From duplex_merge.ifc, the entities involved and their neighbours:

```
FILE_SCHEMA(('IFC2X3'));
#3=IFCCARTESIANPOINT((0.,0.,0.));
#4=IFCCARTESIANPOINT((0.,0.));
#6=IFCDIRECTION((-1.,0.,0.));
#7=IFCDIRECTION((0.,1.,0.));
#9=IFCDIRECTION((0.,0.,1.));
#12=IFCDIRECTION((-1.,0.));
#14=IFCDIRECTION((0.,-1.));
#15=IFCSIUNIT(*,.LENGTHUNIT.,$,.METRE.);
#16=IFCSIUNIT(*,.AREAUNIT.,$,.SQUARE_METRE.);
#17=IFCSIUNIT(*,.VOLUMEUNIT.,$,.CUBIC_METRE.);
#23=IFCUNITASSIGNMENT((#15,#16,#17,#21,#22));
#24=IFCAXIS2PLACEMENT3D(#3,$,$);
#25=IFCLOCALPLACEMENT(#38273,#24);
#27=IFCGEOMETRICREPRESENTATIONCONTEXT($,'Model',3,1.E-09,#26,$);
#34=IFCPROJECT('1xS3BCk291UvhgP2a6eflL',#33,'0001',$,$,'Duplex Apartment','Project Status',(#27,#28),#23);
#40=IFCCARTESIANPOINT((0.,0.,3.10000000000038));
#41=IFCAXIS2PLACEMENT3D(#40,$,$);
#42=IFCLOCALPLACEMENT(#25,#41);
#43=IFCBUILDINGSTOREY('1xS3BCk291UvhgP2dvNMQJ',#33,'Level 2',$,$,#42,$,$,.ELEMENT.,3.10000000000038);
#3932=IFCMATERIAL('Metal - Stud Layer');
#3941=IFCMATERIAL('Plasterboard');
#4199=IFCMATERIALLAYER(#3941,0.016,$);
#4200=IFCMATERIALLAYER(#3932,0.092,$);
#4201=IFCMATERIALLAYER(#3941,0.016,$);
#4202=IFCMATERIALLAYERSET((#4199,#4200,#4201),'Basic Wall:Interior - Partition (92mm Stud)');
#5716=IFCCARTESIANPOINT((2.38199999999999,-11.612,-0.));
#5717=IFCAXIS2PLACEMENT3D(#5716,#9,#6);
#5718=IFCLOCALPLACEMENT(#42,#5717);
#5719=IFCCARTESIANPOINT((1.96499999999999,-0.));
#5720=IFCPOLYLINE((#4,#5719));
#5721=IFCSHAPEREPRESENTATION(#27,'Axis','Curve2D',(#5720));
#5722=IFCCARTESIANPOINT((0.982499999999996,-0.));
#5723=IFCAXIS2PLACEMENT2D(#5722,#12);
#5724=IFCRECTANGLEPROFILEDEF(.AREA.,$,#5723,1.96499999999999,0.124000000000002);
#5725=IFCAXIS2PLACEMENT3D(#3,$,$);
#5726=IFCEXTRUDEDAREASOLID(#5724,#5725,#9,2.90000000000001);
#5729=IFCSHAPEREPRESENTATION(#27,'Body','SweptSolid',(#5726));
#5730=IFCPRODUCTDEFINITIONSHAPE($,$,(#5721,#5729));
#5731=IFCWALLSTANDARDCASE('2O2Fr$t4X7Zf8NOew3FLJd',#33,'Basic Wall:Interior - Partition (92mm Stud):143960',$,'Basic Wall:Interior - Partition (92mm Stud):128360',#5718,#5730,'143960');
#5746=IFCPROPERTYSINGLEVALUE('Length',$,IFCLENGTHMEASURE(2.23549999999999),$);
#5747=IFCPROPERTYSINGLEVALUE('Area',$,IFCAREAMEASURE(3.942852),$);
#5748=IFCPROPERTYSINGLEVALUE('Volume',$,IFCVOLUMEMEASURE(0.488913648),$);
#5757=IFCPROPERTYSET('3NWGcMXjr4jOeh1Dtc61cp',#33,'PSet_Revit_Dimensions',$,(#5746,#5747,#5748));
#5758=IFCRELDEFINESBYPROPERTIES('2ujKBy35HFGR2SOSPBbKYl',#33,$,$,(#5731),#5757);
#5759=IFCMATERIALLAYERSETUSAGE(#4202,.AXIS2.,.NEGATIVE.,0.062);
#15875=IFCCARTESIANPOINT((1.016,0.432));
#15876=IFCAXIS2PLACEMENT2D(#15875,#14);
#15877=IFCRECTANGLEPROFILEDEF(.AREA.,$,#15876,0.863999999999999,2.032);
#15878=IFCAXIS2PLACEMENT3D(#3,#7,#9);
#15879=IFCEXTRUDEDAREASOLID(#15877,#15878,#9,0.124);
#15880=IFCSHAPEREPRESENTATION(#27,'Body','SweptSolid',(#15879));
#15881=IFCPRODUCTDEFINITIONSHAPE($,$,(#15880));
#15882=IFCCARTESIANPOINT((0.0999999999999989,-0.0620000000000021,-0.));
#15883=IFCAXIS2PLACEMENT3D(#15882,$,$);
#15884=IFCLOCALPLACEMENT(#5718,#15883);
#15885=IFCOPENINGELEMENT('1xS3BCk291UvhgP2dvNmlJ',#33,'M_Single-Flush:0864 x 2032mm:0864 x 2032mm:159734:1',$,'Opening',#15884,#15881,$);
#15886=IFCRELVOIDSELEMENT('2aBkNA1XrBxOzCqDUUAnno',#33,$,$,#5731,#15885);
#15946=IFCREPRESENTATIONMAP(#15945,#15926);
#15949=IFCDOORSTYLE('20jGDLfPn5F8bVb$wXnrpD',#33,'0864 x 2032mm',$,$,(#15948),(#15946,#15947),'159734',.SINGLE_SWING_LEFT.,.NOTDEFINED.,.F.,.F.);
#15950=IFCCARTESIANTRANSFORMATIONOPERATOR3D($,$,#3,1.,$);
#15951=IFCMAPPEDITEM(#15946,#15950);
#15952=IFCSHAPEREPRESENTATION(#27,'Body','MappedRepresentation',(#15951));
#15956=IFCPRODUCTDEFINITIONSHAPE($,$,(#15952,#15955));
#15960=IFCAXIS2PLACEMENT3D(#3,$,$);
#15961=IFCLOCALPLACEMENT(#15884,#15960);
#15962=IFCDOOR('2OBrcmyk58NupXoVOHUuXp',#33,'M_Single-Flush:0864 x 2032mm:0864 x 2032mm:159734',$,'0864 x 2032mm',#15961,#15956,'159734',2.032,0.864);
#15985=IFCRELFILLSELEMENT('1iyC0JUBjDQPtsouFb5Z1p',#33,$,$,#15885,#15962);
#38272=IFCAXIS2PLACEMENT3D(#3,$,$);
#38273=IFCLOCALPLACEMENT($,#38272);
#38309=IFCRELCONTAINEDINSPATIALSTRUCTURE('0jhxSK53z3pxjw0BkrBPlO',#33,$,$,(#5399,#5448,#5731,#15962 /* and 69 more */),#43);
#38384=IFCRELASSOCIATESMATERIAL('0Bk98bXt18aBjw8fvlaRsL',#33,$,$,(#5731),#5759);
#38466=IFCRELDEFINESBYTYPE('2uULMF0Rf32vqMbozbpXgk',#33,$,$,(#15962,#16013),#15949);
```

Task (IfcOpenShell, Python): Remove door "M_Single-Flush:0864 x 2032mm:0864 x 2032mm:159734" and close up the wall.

```python
import ifcopenshell
import ifcopenshell.api.feature
import ifcopenshell.api.pset
import ifcopenshell.api.root
import ifcopenshell.geom
import ifcopenshell.util.element
import ifcopenshell.util.shape
import ifcopenshell.util.unit

model = ifcopenshell.open("duplex_merge.ifc")
area_scale = ifcopenshell.util.unit.calculate_unit_scale(model, "AREAUNIT")
volume_scale = ifcopenshell.util.unit.calculate_unit_scale(model, "VOLUMEUNIT")
settings = ifcopenshell.geom.settings()


def volume(element):
    """Net volume in cubic metres, openings subtracted."""
    shape = ifcopenshell.geom.create_shape(settings, element)
    return ifcopenshell.util.shape.get_volume(shape.geometry)


door = model.by_id(15962)
opening = door.FillsVoids[0].RelatingOpeningElement
wall = opening.VoidsElements[0].RelatingBuildingElement
before = volume(wall)

ifcopenshell.api.root.remove_product(model, product=door)
ifcopenshell.api.feature.remove_feature(model, feature=opening)

after = volume(wall)
thickness = 0.124  # wall thickness in metres

# Update the wall's stored quantities.
pset = model.by_id(ifcopenshell.util.element.get_pset(wall, "PSet_Revit_Dimensions", should_inherit=False)["id"])
ifcopenshell.api.pset.edit_pset(model, pset=pset, properties={
    "Area": model.create_entity("IfcAreaMeasure", after / thickness / area_scale),
    "Volume": model.create_entity("IfcVolumeMeasure", after / volume_scale),
})

print(f"wall volume {before:.3f} -> {after:.3f} m3")

model.write("duplex_merge_rev.ifc")
```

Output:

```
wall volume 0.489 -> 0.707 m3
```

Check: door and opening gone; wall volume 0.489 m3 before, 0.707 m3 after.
